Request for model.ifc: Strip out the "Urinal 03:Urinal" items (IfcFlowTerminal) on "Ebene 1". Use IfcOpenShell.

First a look at what the model holds.

```python
import ifcopenshell
import ifcopenshell.util.element

model = ifcopenshell.open("model.ifc")
print(model.schema)
storey = next(s for s in model.by_type("IfcBuildingStorey") if s.Name == "Ebene 1")
terminals = [e for e in ifcopenshell.util.element.get_decomposition(storey) if e.is_a("IfcFlowTerminal")]
seen = {}
for e in terminals:
    element_type = ifcopenshell.util.element.get_type(e)
    name = element_type.Name if element_type not in (None, e) else None
    seen[name] = seen.get(name, 0) + 1
for name, count in sorted(seen.items(), key=str):
    print(count, "x", name)
```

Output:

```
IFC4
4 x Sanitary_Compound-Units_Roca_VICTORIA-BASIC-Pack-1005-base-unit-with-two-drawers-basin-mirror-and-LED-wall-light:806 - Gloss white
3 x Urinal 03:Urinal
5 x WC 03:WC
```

```python
import ifcopenshell
import ifcopenshell.api.root
import ifcopenshell.util.element

model = ifcopenshell.open("model.ifc")

storey = next(s for s in model.by_type("IfcBuildingStorey") if s.Name == "Ebene 1")
terminals = [e for e in ifcopenshell.util.element.get_decomposition(storey) if e.is_a("IfcFlowTerminal")]
targets = [e for e in terminals if (t := ifcopenshell.util.element.get_type(e)) not in (None, e) and t.Name == "Urinal 03:Urinal"]

for e in targets:
    ifcopenshell.api.root.remove_product(model, product=e)
print(len(targets), "removed")

model.write("model_v2.ifc")
```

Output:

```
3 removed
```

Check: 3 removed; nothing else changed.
